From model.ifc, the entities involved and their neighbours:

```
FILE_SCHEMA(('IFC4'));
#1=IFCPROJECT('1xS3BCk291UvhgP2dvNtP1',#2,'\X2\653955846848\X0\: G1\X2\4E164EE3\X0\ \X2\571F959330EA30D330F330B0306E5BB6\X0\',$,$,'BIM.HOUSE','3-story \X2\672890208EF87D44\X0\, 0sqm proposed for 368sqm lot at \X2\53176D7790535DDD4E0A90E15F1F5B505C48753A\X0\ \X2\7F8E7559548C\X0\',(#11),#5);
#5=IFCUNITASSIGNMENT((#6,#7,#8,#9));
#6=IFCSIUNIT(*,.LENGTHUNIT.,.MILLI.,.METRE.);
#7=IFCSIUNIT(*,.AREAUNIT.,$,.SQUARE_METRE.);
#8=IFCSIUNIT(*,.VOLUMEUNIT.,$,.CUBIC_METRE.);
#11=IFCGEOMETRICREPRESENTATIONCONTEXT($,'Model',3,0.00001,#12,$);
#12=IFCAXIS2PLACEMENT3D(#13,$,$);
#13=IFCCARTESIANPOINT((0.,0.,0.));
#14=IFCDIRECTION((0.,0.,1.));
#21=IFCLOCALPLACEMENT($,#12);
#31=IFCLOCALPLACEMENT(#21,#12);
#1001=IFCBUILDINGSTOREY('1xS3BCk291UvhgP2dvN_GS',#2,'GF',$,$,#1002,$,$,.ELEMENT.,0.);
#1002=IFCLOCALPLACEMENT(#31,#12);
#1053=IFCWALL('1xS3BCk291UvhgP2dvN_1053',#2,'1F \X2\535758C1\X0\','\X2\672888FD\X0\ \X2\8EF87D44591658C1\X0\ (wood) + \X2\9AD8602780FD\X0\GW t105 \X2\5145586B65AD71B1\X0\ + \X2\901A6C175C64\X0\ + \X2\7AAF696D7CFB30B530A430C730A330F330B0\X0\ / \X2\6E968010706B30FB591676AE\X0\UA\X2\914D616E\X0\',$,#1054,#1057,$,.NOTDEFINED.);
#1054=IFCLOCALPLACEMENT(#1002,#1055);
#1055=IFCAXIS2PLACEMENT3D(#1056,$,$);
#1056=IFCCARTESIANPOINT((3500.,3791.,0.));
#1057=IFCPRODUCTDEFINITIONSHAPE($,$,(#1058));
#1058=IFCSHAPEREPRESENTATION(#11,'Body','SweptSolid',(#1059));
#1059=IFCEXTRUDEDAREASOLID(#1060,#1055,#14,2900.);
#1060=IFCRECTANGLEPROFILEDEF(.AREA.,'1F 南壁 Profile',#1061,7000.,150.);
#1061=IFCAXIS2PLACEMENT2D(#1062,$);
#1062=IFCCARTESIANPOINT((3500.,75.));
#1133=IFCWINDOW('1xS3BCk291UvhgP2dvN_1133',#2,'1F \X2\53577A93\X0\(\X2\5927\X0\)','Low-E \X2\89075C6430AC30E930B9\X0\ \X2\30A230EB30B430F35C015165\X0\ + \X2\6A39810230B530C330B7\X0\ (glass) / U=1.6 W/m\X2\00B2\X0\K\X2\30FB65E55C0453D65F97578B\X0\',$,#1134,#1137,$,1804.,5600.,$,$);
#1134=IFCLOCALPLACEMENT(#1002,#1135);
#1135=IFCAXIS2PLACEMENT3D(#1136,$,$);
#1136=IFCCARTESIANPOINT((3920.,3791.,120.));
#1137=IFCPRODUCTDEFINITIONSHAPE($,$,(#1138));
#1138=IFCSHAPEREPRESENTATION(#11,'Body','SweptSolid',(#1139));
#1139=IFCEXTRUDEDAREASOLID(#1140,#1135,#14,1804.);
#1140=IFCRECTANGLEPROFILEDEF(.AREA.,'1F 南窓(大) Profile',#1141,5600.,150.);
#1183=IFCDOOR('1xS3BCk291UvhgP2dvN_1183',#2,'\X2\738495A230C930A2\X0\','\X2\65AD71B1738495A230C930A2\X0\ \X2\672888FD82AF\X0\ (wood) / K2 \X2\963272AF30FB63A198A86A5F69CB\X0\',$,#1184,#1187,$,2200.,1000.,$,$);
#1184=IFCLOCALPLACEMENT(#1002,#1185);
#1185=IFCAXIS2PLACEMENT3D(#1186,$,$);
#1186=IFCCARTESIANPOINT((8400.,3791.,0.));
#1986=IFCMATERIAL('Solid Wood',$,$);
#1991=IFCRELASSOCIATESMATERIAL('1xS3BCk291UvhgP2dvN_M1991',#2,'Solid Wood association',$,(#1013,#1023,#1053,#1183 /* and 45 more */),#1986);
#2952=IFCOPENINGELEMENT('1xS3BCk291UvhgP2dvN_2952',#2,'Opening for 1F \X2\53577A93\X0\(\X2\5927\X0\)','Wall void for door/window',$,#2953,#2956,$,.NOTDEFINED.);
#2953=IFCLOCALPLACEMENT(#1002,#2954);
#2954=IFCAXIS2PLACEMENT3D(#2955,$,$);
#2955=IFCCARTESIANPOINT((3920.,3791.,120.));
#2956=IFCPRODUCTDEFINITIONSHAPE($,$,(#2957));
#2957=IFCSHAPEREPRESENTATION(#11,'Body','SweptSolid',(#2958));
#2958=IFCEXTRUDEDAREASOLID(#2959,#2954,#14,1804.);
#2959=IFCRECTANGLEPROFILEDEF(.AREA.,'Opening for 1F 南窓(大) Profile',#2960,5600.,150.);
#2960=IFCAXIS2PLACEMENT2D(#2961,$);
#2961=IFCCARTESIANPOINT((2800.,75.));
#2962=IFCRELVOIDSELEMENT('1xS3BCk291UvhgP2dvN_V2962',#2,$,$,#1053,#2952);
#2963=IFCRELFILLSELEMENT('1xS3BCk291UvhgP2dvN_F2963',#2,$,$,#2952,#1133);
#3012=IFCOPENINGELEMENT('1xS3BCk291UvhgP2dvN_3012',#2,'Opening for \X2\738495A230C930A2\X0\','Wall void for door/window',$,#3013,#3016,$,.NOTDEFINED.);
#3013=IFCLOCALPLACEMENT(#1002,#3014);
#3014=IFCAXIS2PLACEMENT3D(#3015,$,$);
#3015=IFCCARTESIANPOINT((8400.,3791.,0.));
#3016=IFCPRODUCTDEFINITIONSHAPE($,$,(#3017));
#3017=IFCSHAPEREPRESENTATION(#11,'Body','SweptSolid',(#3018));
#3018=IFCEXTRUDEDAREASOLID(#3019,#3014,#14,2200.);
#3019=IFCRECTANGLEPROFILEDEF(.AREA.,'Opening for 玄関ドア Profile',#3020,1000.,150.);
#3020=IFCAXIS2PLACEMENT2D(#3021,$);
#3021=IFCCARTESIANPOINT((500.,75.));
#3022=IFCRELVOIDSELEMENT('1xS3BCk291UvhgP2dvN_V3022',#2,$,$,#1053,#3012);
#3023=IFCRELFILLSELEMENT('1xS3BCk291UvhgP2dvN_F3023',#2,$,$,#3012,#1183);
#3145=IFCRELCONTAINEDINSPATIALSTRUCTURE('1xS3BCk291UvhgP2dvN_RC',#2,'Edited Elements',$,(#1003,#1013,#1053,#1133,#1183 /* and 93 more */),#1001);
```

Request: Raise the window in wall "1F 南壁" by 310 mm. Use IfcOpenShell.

```python
import numpy as np
import ifcopenshell
import ifcopenshell.api.geometry
import ifcopenshell.util.placement
import ifcopenshell.util.unit

model = ifcopenshell.open("model.ifc")
unit_scale = ifcopenshell.util.unit.calculate_unit_scale(model)

window = model.by_id(1133)
opening = window.FillsVoids[0].RelatingOpeningElement
dz = 310.0

shift = np.array([0.0, 0.0, dz])
# The window is not placed relative to its opening, so move both.
for product in (opening, window):
    matrix = ifcopenshell.util.placement.get_local_placement(product.ObjectPlacement)
    matrix[:3, 3] += shift
    ifcopenshell.api.geometry.edit_object_placement(model, product=product, matrix=matrix, is_si=False)

print(f"moved by {dz * unit_scale:+.3f} m")

model.write("model-out.ifc")
```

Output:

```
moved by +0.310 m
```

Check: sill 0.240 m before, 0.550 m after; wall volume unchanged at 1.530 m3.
